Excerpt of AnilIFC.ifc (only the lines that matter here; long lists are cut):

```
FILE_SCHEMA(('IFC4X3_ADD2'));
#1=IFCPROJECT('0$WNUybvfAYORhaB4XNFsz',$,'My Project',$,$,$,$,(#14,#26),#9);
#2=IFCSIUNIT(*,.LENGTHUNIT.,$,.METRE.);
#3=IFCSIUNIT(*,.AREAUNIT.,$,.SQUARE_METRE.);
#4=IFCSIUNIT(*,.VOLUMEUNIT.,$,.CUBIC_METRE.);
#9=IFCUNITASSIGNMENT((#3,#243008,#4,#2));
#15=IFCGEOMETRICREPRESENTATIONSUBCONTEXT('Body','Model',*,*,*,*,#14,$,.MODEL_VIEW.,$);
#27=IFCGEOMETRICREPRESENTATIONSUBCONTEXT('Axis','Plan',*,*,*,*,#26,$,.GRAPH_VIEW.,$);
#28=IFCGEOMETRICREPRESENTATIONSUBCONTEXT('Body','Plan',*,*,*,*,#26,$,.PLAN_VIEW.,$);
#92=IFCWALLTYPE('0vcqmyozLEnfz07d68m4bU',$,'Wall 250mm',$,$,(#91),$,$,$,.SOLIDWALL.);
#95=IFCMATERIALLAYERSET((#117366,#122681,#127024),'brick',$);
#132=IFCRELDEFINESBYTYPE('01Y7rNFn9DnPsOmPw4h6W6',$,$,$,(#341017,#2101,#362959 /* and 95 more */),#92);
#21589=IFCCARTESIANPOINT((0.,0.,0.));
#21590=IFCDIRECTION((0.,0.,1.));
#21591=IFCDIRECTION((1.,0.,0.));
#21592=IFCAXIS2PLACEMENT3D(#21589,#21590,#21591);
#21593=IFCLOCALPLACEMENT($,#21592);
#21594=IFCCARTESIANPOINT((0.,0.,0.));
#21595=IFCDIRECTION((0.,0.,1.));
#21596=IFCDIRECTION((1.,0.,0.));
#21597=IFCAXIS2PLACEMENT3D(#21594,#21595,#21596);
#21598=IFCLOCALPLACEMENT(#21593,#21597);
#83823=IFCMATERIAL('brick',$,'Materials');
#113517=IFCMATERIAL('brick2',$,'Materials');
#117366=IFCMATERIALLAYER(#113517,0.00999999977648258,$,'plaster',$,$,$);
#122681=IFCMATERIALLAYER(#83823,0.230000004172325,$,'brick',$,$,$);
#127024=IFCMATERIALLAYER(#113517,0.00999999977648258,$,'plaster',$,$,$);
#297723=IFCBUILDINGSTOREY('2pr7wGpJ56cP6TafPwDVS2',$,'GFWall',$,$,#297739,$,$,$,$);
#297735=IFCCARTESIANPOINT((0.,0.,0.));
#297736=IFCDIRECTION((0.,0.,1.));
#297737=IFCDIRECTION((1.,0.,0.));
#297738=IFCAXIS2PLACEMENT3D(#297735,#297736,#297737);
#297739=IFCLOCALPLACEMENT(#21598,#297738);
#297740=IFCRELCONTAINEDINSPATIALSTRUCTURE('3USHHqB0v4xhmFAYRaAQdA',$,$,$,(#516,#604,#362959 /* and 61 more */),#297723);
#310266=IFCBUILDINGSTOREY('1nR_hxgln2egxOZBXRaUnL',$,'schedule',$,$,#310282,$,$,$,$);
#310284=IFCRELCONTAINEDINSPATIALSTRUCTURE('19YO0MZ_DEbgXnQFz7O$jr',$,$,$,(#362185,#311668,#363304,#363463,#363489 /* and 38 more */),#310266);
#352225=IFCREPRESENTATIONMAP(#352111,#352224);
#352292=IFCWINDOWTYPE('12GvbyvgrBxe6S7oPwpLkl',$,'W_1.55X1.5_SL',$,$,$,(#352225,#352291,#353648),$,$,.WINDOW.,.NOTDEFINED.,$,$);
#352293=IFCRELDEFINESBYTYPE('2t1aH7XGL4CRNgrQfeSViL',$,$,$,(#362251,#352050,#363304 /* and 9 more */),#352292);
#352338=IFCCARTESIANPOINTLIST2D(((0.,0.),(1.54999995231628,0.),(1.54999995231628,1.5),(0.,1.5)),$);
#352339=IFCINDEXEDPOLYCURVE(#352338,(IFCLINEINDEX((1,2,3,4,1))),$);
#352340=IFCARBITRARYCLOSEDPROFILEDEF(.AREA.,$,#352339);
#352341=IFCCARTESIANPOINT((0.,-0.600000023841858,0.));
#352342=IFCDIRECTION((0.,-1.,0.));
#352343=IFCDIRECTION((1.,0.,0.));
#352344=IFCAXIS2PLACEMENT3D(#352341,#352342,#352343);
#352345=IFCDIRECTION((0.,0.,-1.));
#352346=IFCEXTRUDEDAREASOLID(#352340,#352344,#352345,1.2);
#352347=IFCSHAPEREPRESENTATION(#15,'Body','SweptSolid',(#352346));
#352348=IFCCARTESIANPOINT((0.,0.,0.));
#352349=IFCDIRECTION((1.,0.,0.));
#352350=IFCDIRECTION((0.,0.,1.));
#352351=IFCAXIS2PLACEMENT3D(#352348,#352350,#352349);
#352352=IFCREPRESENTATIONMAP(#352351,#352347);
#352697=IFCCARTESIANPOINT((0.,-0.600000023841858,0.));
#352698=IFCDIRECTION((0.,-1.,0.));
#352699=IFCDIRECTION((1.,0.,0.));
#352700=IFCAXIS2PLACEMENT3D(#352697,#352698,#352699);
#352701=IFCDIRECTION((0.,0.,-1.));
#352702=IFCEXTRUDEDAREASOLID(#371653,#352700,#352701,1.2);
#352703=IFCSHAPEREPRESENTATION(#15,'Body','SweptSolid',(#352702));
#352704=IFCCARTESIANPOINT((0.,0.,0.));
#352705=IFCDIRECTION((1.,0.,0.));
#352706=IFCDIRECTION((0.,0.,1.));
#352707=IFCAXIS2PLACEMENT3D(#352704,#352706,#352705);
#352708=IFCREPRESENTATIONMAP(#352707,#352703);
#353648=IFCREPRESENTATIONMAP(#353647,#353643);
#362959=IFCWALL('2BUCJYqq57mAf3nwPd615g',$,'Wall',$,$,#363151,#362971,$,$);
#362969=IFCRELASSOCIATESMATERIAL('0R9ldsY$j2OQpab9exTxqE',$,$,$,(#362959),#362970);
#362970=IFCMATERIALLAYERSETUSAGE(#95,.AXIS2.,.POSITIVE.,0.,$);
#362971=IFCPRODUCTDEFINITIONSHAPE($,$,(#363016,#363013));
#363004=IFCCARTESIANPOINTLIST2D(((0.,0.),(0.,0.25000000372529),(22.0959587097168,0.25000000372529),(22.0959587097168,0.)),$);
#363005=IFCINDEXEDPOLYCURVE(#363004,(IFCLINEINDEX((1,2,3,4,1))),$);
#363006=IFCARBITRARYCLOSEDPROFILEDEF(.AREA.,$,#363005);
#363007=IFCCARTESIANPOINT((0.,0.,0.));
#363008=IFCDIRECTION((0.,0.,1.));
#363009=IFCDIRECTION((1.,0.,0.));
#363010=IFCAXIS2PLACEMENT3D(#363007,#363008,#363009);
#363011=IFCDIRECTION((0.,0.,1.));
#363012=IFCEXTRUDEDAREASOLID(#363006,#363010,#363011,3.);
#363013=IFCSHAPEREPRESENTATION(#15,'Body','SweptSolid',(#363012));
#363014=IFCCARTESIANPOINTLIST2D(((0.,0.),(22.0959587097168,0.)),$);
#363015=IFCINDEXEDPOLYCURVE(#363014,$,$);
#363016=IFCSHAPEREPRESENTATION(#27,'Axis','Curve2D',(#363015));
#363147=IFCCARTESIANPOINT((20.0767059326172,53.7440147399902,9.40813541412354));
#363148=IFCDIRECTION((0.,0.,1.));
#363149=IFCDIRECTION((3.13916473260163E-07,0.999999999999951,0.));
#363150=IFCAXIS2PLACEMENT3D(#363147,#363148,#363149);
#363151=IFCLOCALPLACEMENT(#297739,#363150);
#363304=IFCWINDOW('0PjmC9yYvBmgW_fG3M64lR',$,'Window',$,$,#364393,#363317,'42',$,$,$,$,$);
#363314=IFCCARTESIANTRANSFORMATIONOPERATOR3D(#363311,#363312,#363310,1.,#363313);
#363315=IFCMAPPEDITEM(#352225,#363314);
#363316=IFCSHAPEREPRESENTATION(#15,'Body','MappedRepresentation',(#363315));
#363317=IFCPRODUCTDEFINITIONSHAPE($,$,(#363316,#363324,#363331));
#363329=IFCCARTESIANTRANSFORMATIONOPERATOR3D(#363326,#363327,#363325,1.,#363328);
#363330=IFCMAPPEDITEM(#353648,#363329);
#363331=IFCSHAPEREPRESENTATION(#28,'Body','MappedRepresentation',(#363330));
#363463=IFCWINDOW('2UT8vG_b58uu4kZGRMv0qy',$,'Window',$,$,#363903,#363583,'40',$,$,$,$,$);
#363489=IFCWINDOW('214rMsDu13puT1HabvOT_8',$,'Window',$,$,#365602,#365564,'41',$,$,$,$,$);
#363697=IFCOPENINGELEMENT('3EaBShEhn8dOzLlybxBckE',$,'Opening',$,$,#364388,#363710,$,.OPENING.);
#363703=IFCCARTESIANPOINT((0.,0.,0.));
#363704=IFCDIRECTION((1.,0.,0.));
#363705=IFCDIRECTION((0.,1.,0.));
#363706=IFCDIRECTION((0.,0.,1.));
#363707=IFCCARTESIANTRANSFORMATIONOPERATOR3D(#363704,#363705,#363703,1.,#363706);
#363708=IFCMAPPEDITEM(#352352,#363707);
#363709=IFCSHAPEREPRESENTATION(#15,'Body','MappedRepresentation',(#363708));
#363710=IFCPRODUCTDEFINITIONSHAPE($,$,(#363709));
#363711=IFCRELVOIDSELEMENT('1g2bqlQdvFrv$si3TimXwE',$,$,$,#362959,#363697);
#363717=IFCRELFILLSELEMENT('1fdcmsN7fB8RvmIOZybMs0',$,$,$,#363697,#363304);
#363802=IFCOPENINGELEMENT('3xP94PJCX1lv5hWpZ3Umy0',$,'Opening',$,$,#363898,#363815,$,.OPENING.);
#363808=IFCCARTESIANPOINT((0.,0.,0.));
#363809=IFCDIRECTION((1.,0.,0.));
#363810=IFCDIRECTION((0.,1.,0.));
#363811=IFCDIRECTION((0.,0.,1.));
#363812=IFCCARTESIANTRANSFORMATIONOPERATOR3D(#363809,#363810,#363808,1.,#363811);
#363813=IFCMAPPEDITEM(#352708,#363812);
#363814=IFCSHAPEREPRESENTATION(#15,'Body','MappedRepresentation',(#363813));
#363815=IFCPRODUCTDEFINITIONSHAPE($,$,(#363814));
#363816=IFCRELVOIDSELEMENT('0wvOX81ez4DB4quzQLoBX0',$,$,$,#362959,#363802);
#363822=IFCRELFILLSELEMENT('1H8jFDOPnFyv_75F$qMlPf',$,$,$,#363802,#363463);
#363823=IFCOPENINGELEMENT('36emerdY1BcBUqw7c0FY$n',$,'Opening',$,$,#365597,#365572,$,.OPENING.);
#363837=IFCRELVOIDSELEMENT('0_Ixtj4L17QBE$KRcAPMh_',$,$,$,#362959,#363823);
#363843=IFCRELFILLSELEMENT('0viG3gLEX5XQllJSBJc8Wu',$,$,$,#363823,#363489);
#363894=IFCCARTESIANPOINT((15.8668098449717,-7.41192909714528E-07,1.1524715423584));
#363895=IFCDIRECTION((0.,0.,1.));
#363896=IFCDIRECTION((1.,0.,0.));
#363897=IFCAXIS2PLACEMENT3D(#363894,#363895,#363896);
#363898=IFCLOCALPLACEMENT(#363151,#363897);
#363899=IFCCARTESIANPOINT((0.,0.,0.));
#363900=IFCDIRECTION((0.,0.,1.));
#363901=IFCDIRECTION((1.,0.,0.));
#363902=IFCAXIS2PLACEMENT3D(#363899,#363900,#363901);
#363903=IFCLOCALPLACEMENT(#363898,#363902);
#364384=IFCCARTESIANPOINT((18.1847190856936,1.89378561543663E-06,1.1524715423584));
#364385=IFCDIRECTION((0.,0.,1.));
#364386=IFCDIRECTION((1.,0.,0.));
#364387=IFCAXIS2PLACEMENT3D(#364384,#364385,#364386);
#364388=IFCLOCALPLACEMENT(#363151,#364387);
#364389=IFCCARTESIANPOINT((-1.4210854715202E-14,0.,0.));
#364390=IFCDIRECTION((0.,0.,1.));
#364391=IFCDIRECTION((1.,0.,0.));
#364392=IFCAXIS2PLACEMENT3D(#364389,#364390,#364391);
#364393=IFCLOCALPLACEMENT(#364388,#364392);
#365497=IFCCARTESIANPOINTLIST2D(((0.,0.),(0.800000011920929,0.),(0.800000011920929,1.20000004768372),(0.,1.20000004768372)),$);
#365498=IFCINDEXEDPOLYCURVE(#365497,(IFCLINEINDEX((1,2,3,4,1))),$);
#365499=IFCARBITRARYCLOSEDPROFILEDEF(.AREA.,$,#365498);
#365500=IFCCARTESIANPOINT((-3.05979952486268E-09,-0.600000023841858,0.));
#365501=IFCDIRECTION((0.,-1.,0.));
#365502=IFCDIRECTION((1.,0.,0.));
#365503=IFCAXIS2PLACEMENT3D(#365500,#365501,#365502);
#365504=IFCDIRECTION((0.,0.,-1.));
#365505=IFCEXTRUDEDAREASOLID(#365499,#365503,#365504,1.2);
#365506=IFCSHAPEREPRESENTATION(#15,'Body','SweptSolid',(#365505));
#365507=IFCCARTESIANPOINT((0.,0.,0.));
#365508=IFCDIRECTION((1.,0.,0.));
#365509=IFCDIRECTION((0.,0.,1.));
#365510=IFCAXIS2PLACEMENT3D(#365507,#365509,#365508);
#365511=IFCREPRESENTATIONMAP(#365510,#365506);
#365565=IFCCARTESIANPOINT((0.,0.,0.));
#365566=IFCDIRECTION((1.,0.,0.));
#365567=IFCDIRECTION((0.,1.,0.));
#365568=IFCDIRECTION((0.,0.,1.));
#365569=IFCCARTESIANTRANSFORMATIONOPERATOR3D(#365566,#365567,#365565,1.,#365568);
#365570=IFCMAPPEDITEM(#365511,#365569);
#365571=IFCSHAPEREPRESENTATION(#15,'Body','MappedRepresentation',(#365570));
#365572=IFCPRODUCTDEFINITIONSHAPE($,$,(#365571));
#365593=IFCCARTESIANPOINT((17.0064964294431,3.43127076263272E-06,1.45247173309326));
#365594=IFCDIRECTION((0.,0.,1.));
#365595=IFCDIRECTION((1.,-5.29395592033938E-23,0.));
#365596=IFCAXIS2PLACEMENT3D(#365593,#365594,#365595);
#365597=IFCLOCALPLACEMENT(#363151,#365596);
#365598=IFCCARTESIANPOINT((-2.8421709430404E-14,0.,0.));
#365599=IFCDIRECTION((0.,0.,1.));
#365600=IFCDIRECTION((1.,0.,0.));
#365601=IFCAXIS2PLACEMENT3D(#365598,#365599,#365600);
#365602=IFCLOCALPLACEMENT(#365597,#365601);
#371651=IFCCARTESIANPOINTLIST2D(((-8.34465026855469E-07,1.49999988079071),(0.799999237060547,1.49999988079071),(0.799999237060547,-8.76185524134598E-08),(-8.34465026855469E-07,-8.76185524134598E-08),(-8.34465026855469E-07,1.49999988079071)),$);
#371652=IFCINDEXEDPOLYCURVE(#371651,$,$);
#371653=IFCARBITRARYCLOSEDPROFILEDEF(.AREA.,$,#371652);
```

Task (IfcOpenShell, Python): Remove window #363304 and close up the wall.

```python
import ifcopenshell
import ifcopenshell.api.feature
import ifcopenshell.api.root
import ifcopenshell.geom
import ifcopenshell.util.shape

model = ifcopenshell.open("AnilIFC.ifc")
settings = ifcopenshell.geom.settings()


def volume(element):
    """Net volume in cubic metres, openings subtracted."""
    shape = ifcopenshell.geom.create_shape(settings, element)
    return ifcopenshell.util.shape.get_volume(shape.geometry)


window = model.by_id(363304)
opening = window.FillsVoids[0].RelatingOpeningElement
wall = opening.VoidsElements[0].RelatingBuildingElement
before = volume(wall)

ifcopenshell.api.root.remove_product(model, product=window)
ifcopenshell.api.feature.remove_feature(model, feature=opening)

after = volume(wall)

print(f"wall volume {before:.3f} -> {after:.3f} m3")

model.write("AnilIFC_edited.ifc")
```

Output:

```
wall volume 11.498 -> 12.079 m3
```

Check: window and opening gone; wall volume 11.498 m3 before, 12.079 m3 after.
